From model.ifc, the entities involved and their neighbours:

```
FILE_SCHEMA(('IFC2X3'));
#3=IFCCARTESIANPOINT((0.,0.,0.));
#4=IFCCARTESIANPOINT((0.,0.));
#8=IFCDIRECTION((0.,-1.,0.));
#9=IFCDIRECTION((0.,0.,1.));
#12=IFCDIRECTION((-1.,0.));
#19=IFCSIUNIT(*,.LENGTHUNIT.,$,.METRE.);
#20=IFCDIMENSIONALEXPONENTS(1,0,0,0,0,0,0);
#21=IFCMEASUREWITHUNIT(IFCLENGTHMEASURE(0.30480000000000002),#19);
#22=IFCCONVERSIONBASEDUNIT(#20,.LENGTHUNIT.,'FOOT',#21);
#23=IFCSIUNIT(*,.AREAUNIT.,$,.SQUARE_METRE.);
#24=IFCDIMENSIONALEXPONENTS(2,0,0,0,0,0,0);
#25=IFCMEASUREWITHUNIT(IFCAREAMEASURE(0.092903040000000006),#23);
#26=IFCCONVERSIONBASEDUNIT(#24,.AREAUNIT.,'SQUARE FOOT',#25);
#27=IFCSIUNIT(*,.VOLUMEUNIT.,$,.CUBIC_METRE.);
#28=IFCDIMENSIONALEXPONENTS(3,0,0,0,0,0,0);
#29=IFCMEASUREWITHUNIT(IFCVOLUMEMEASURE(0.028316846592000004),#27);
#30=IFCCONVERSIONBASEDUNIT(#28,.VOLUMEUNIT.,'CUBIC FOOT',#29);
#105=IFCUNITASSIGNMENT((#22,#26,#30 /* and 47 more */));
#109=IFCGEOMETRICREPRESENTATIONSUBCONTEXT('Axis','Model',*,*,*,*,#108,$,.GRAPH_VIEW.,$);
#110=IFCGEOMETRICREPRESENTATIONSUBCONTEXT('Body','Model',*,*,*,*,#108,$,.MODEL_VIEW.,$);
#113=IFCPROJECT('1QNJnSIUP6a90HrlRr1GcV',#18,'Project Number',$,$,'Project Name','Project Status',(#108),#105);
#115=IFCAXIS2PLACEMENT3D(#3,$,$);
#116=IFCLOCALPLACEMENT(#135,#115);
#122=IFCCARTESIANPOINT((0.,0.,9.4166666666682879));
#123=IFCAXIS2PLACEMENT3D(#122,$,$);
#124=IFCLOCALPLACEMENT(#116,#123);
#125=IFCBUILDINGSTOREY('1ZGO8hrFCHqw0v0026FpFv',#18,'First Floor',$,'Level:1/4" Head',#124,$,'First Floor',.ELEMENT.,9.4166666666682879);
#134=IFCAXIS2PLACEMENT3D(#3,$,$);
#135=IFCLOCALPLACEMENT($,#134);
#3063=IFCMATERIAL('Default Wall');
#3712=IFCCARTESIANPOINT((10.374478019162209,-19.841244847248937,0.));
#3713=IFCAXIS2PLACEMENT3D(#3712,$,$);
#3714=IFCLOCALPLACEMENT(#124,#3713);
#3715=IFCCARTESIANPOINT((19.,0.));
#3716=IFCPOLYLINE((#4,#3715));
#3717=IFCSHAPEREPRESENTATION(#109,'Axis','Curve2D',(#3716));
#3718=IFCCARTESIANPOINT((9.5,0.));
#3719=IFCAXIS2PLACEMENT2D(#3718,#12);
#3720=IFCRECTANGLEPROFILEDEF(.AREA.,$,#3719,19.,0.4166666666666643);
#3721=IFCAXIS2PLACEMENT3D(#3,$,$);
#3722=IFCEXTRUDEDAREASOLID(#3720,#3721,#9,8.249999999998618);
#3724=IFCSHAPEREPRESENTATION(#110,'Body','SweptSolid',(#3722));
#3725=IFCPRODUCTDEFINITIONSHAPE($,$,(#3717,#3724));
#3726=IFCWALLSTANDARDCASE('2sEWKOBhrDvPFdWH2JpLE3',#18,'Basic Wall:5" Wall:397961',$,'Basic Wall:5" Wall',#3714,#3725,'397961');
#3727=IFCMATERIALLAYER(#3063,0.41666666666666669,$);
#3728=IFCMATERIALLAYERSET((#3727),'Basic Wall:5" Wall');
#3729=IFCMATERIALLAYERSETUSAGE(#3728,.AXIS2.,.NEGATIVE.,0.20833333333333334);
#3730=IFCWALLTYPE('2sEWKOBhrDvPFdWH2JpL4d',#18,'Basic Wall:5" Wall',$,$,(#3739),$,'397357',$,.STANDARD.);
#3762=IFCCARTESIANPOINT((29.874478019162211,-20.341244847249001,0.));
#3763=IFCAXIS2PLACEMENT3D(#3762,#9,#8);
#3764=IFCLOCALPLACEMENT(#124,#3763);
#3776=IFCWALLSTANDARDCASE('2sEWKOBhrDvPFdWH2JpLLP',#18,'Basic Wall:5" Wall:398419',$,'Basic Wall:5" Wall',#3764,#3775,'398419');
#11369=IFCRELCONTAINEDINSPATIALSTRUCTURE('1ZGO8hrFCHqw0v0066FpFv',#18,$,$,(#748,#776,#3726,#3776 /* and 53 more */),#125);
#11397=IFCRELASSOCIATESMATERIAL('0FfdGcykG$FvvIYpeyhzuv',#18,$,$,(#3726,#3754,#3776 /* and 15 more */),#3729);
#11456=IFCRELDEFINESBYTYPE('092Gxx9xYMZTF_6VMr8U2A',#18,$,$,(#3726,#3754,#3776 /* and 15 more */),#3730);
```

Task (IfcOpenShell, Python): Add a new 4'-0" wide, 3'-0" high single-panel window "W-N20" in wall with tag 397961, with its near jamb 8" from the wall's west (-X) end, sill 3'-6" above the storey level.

```python
import numpy as np
import ifcopenshell
import ifcopenshell.api.feature
import ifcopenshell.api.geometry
import ifcopenshell.api.root
import ifcopenshell.api.spatial
import ifcopenshell.api.type
import ifcopenshell.geom
import ifcopenshell.util.element
import ifcopenshell.util.placement
import ifcopenshell.util.representation
import ifcopenshell.util.shape
import ifcopenshell.util.unit

model = ifcopenshell.open("model.ifc")
unit_scale = ifcopenshell.util.unit.calculate_unit_scale(model)
settings = ifcopenshell.geom.settings()


def volume(element):
    """Net volume in cubic metres, openings subtracted."""
    shape = ifcopenshell.geom.create_shape(settings, element)
    return ifcopenshell.util.shape.get_volume(shape.geometry)


wall = model.by_guid("2sEWKOBhrDvPFdWH2JpLE3")
storey = ifcopenshell.util.element.get_container(wall, ifc_class="IfcBuildingStorey")
context = ifcopenshell.util.representation.get_context(model, "Model", "Body", "MODEL_VIEW")
before = volume(wall)

width, height, from_end, sill = 1.2192, 0.9144, 0.2032, 1.0668  # metres

# The wall runs along its own X axis, and the end named is its -X end.
wall_shape = ifcopenshell.geom.create_shape(settings, wall)
x, y, z = ifcopenshell.util.shape.get_vertices(wall_shape.geometry).T
start = x.min() + from_end
face, thickness = float(y.min()), float(y.max() - y.min())
wall_matrix = ifcopenshell.util.placement.get_local_placement(wall.ObjectPlacement)
level = ifcopenshell.util.placement.get_local_placement(storey.ObjectPlacement)[2, 3]


def in_wall(x, y):
    """Placement at x, y metres in the wall's axes, at sill height."""
    matrix = wall_matrix.copy()
    matrix[:, 3] = wall_matrix @ np.array([x / unit_scale, y / unit_scale, 0.0, 1.0])
    matrix[2, 3] = level + sill / unit_scale
    return matrix


# Opening: a box that overshoots both wall faces by 50 mm.
opening = ifcopenshell.api.root.create_entity(model, ifc_class="IfcOpeningElement")
box = ifcopenshell.api.geometry.add_wall_representation(
    model, context=context, length=width, height=height, thickness=thickness + 0.1
)
ifcopenshell.api.geometry.assign_representation(model, product=opening, representation=box)
ifcopenshell.api.geometry.edit_object_placement(model, product=opening, matrix=in_wall(start, face - 0.05), is_si=False)
ifcopenshell.api.feature.add_feature(model, feature=opening, element=wall)

window = ifcopenshell.api.root.create_entity(model, ifc_class="IfcWindow", name="W-N20")
window.OverallWidth, window.OverallHeight = width / unit_scale, height / unit_scale
body = ifcopenshell.api.geometry.add_window_representation(
    model,
    context=context,
    overall_width=window.OverallWidth,
    overall_height=window.OverallHeight,
    partition_type="SINGLE_PANEL",
)
ifcopenshell.api.geometry.assign_representation(model, product=window, representation=body)
ifcopenshell.api.spatial.assign_container(model, products=[window], relating_structure=storey)
fills = ifcopenshell.api.feature.add_filling(model, opening=opening, element=window)
fills.OwnerHistory = window.OwnerHistory  # required in IFC2X3

# IFC2X3 keeps the operation on the window style.
style = ifcopenshell.api.root.create_entity(model, ifc_class="IfcWindowStyle", name="W-N20")
style.OperationType, style.ConstructionType = "SINGLE_PANEL", "NOTDEFINED"
style.ParameterTakesPrecedence = style.Sizeable = False
ifcopenshell.api.type.assign_type(model, related_objects=[window], relating_type=style)

# Centre the window in the wall's thickness.
ifcopenshell.api.geometry.edit_object_placement(model, product=window, matrix=in_wall(start, face), is_si=False)
window_shape = ifcopenshell.geom.create_shape(settings, window)
depth = ifcopenshell.util.shape.get_vertices(window_shape.geometry)[:, 1]
offset = face + thickness / 2 - (depth.min() + depth.max()) / 2
ifcopenshell.api.geometry.edit_object_placement(model, product=window, matrix=in_wall(start, offset), is_si=False)

after = volume(wall)

print(f"wall volume {before:.3f} -> {after:.3f} m3")

model.write("model_v2.ifc")
```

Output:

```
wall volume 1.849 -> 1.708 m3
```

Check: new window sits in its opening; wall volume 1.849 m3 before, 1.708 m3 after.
